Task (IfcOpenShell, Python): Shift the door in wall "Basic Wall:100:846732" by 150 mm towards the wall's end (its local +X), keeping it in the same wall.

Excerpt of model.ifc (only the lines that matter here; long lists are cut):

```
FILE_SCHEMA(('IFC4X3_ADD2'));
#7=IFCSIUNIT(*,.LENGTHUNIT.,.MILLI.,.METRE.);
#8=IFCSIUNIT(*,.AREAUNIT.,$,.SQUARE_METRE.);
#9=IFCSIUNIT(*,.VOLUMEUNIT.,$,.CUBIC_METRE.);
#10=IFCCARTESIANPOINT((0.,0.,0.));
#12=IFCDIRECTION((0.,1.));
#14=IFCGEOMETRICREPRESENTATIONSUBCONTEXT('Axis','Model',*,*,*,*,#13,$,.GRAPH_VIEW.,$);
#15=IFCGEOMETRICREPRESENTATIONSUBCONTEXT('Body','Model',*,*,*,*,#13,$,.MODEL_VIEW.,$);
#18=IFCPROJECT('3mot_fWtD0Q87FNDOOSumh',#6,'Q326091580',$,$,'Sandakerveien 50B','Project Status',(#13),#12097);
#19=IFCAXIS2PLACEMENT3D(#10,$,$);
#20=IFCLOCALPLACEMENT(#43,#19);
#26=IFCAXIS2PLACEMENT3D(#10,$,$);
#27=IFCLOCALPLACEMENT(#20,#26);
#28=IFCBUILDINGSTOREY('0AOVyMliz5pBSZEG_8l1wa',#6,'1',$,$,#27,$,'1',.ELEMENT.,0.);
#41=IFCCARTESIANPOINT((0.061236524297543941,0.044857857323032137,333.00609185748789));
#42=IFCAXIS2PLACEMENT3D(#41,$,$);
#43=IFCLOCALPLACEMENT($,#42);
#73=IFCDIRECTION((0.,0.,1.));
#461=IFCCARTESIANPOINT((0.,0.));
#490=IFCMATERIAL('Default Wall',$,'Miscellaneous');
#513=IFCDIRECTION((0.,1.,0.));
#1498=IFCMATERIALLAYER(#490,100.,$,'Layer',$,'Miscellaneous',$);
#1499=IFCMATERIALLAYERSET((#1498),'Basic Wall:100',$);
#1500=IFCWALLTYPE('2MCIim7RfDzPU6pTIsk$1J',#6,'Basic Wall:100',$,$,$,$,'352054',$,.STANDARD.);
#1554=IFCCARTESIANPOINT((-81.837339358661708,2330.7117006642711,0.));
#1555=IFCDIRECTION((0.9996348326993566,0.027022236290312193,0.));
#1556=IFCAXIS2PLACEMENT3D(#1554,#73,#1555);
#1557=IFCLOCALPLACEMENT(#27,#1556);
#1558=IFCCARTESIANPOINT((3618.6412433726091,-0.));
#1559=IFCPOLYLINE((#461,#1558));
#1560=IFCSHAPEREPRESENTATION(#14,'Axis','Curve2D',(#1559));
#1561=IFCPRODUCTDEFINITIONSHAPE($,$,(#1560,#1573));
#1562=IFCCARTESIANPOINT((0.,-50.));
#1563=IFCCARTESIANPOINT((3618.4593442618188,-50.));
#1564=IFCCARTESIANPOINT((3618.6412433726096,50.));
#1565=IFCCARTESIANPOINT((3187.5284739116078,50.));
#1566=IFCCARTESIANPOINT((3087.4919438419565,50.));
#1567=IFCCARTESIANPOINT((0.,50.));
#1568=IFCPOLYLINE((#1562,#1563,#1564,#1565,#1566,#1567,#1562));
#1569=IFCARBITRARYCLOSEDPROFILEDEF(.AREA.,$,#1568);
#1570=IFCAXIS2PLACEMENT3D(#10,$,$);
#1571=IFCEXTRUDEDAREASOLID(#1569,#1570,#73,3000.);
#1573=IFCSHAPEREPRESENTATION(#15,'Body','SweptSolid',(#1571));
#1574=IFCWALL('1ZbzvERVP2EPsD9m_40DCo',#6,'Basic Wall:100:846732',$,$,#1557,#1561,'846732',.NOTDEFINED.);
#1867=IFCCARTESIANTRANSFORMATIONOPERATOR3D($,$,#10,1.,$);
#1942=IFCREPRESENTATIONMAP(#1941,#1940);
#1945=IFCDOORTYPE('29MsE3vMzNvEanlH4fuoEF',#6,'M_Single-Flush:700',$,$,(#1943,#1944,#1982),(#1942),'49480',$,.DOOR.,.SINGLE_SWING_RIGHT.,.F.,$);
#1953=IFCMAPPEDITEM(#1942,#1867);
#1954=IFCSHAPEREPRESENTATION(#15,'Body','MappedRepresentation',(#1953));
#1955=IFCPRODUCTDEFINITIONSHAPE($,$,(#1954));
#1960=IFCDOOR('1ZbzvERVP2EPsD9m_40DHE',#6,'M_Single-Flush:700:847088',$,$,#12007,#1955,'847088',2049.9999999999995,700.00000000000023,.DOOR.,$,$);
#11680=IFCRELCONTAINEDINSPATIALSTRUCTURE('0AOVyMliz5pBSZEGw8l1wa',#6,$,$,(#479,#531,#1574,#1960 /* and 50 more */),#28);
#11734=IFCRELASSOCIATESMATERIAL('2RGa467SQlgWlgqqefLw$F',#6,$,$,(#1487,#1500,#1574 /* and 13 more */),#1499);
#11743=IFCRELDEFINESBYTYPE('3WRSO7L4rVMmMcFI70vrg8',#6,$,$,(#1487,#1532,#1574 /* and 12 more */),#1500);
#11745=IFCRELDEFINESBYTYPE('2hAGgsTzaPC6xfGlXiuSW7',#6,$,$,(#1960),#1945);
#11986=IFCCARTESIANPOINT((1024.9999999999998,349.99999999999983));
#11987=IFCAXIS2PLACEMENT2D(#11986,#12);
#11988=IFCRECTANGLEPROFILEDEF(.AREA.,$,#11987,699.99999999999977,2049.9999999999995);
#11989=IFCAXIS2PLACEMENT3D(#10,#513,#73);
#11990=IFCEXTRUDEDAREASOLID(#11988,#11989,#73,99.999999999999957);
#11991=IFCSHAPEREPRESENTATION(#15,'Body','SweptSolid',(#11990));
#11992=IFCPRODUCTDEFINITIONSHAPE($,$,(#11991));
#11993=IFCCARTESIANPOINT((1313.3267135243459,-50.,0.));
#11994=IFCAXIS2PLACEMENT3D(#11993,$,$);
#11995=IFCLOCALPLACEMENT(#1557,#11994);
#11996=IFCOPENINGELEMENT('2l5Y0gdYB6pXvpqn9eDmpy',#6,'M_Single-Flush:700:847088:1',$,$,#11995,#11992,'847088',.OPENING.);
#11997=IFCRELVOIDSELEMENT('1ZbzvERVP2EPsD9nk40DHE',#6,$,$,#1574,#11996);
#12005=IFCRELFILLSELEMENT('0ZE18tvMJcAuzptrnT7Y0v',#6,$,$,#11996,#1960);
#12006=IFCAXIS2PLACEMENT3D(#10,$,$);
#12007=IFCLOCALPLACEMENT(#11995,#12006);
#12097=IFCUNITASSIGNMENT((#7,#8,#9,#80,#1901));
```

```python
import ifcopenshell
import ifcopenshell.api.geometry
import ifcopenshell.util.placement
import ifcopenshell.util.unit

model = ifcopenshell.open("model.ifc")
unit_scale = ifcopenshell.util.unit.calculate_unit_scale(model)

door = model.by_guid("1ZbzvERVP2EPsD9m_40DHE")
opening = door.FillsVoids[0].RelatingOpeningElement
wall = opening.VoidsElements[0].RelatingBuildingElement

wall_matrix = ifcopenshell.util.placement.get_local_placement(wall.ObjectPlacement)
shift = wall_matrix[:3, 0] * 0.15 / unit_scale
before = ifcopenshell.util.placement.get_local_placement(door.ObjectPlacement)[:3, 3].copy()

# The door is placed relative to its opening, so it follows when the opening moves.
matrix = ifcopenshell.util.placement.get_local_placement(opening.ObjectPlacement)
matrix[:3, 3] += shift
ifcopenshell.api.geometry.edit_object_placement(
    model, product=opening, matrix=matrix, is_si=False, should_transform_children=True
)

after = ifcopenshell.util.placement.get_local_placement(door.ObjectPlacement)[:3, 3]
print("door moved by", (after - before).round(3) + 0.0)

model.write("model-out.ifc")
```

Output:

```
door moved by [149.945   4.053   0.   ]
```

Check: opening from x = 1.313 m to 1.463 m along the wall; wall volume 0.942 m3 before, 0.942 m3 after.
